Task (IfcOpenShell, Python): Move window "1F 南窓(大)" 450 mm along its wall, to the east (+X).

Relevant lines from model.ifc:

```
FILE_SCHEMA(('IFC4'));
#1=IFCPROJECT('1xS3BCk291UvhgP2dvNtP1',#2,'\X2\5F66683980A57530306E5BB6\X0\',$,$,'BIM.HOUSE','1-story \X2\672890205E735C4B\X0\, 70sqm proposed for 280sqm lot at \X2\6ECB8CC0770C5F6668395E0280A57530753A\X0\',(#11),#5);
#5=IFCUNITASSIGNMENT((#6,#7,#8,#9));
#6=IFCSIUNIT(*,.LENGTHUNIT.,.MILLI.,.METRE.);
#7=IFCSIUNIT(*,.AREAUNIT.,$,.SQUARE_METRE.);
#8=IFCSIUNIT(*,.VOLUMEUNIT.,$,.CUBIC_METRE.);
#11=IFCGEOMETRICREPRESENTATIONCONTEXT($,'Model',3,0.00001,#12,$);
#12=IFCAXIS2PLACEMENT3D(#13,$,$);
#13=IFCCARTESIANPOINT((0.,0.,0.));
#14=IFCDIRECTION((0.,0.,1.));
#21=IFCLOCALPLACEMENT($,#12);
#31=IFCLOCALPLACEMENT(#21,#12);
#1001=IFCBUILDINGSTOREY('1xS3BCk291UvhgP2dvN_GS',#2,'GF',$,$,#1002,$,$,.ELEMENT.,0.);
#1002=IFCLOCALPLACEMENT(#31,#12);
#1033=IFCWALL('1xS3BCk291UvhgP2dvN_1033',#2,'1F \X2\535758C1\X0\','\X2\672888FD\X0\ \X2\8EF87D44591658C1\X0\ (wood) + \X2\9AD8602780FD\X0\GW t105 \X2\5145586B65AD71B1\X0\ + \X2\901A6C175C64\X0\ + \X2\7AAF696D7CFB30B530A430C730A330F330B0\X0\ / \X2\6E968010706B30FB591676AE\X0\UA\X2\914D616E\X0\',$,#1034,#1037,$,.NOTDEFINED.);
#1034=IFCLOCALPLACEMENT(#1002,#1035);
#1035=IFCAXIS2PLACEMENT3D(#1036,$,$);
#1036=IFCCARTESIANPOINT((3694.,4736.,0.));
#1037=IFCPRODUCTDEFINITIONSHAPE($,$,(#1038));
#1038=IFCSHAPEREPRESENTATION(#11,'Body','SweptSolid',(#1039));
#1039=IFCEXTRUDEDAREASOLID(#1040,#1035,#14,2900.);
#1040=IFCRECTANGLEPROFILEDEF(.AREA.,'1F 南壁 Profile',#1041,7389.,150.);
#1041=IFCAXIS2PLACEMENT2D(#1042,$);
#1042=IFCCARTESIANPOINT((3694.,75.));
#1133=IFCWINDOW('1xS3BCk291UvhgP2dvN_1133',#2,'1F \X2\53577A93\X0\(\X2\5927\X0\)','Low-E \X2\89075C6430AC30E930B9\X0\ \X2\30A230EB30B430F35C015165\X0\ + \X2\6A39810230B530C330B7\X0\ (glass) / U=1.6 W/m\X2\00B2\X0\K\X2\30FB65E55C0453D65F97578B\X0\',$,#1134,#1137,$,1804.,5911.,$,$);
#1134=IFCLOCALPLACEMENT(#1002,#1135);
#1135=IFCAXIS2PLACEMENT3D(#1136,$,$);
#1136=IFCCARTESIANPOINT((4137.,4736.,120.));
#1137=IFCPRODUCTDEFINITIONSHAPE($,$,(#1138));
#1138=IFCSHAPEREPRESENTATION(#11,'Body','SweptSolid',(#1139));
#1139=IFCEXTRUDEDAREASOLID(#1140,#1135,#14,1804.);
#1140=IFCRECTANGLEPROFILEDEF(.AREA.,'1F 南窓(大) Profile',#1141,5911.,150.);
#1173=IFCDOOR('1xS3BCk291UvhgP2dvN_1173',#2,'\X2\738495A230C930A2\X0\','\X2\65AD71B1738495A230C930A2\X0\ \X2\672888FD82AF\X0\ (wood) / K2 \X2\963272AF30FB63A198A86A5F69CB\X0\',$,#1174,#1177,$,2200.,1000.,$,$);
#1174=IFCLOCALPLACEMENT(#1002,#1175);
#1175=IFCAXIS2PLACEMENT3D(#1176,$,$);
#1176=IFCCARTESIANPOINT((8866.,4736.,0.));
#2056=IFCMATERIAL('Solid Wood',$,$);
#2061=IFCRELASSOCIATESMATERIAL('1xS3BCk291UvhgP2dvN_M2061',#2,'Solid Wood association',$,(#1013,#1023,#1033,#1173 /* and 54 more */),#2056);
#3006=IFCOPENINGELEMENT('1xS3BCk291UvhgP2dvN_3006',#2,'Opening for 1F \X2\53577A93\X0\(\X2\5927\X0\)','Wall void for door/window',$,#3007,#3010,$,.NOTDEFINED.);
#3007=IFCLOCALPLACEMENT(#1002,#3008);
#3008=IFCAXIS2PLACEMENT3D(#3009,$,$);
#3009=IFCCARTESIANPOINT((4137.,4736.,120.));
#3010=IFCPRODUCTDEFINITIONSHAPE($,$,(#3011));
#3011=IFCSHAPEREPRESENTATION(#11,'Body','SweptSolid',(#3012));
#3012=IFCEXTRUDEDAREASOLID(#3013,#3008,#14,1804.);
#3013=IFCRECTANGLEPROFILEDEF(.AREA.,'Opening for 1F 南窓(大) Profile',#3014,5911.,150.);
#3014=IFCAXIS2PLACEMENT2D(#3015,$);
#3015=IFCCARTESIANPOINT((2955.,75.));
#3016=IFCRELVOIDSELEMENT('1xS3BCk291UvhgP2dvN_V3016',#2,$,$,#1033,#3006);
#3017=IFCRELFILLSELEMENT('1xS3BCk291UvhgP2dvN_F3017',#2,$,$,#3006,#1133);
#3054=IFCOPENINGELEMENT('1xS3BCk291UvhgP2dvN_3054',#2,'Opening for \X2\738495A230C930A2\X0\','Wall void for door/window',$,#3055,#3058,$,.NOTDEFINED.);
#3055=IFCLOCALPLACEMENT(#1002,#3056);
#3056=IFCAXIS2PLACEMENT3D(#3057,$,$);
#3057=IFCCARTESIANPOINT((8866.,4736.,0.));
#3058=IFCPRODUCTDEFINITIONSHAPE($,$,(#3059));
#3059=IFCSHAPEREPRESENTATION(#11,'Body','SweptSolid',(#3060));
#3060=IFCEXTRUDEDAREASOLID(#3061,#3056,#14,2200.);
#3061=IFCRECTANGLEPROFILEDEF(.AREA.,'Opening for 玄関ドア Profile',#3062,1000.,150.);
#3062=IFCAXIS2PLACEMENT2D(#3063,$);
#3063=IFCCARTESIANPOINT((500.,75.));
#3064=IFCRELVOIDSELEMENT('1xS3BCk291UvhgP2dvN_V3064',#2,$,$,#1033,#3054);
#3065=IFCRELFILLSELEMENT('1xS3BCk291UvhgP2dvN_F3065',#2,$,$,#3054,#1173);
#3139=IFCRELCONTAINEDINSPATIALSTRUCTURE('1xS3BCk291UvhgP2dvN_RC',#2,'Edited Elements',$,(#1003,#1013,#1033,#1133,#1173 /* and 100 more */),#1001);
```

```python
import ifcopenshell
import ifcopenshell.api.geometry
import ifcopenshell.util.placement
import ifcopenshell.util.unit

model = ifcopenshell.open("model.ifc")
unit_scale = ifcopenshell.util.unit.calculate_unit_scale(model)

window = model.by_guid("1xS3BCk291UvhgP2dvN_1133")
opening = window.FillsVoids[0].RelatingOpeningElement
wall = opening.VoidsElements[0].RelatingBuildingElement

wall_matrix = ifcopenshell.util.placement.get_local_placement(wall.ObjectPlacement)
shift = wall_matrix[:3, 0] * 0.45 / unit_scale
before = ifcopenshell.util.placement.get_local_placement(window.ObjectPlacement)[:3, 3].copy()

# The window is not placed relative to its opening, so move both.
for product in (opening, window):
    matrix = ifcopenshell.util.placement.get_local_placement(product.ObjectPlacement)
    matrix[:3, 3] += shift
    ifcopenshell.api.geometry.edit_object_placement(model, product=product, matrix=matrix, is_si=False)

after = ifcopenshell.util.placement.get_local_placement(window.ObjectPlacement)[:3, 3]
print("window moved by", (after - before).round(3) + 0.0)

model.write("model_updated.ifc")
```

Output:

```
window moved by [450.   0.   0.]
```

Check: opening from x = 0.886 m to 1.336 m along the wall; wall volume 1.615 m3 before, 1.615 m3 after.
